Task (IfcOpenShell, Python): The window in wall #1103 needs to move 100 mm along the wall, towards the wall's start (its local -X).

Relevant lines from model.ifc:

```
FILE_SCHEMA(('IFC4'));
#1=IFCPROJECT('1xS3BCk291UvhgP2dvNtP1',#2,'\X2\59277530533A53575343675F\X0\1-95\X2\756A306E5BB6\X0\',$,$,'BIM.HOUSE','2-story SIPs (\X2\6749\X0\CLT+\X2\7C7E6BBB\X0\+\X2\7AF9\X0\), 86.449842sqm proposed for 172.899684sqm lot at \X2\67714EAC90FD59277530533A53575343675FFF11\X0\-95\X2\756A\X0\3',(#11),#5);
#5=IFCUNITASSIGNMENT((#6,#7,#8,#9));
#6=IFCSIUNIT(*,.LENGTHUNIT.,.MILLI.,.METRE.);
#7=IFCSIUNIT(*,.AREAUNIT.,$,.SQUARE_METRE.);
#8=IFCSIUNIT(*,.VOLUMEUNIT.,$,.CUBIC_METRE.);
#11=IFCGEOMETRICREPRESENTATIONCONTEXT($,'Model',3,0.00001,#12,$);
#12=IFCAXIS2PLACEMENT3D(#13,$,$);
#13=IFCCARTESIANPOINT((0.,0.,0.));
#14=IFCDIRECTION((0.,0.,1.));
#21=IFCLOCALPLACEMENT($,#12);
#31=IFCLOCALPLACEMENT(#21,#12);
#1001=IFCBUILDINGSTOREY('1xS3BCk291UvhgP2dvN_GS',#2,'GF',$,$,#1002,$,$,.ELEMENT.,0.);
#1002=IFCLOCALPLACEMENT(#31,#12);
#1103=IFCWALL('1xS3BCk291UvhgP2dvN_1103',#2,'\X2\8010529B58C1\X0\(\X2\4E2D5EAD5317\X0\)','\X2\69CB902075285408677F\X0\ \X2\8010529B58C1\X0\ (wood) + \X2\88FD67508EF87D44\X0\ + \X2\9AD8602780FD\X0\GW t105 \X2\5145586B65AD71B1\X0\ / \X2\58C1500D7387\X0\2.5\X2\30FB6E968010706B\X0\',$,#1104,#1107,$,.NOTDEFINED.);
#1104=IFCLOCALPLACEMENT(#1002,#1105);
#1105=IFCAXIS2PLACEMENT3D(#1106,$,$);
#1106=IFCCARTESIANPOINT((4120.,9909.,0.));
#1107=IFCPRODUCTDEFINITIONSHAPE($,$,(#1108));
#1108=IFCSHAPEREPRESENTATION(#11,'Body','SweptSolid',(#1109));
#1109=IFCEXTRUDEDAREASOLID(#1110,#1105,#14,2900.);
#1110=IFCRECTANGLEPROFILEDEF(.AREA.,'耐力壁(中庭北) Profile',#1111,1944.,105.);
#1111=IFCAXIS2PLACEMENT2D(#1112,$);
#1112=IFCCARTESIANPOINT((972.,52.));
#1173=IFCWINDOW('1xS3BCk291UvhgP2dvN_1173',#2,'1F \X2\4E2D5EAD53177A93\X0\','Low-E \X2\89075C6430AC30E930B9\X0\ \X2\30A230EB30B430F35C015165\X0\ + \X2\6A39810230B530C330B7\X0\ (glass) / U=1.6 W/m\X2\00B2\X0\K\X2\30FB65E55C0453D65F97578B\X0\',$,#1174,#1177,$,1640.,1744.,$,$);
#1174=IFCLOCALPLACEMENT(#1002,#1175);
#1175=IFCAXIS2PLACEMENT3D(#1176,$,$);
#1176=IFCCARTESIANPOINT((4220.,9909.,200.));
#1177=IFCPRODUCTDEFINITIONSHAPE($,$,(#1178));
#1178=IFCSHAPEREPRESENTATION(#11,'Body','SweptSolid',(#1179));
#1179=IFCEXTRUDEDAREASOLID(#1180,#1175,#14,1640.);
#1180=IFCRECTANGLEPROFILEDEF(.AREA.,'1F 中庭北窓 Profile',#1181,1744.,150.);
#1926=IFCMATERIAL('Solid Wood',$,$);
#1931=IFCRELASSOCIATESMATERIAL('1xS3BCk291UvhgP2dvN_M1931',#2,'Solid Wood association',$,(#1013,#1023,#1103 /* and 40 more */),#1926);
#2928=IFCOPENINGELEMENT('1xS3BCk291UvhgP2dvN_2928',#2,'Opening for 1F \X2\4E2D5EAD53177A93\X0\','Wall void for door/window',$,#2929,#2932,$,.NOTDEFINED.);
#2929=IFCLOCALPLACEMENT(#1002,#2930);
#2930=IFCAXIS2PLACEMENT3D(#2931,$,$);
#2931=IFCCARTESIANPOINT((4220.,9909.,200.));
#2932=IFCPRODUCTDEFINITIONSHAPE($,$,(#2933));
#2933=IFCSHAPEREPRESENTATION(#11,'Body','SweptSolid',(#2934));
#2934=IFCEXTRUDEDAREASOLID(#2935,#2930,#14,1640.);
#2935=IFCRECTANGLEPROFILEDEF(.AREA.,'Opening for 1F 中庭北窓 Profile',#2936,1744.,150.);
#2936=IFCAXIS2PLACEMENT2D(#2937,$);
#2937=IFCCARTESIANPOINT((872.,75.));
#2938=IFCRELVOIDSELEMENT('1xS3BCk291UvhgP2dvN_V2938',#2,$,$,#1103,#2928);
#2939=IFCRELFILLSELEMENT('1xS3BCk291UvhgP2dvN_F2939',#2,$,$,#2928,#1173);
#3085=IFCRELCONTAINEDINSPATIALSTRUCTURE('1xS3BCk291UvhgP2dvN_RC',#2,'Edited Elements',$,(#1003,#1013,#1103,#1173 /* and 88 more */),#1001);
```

```python
import ifcopenshell
import ifcopenshell.api.geometry
import ifcopenshell.util.placement
import ifcopenshell.util.unit

model = ifcopenshell.open("model.ifc")
unit_scale = ifcopenshell.util.unit.calculate_unit_scale(model)

window = model.by_guid("1xS3BCk291UvhgP2dvN_1173")
opening = window.FillsVoids[0].RelatingOpeningElement
wall = opening.VoidsElements[0].RelatingBuildingElement

wall_matrix = ifcopenshell.util.placement.get_local_placement(wall.ObjectPlacement)
shift = wall_matrix[:3, 0] * -0.1 / unit_scale
before = ifcopenshell.util.placement.get_local_placement(window.ObjectPlacement)[:3, 3].copy()

# The window is not placed relative to its opening, so move both.
for product in (opening, window):
    matrix = ifcopenshell.util.placement.get_local_placement(product.ObjectPlacement)
    matrix[:3, 3] += shift
    ifcopenshell.api.geometry.edit_object_placement(model, product=product, matrix=matrix, is_si=False)

after = ifcopenshell.util.placement.get_local_placement(window.ObjectPlacement)[:3, 3]
print("window moved by", (after - before).round(3) + 0.0)

model.write("model_updated.ifc")
```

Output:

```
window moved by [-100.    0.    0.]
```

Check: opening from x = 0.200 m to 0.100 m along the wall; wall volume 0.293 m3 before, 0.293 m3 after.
